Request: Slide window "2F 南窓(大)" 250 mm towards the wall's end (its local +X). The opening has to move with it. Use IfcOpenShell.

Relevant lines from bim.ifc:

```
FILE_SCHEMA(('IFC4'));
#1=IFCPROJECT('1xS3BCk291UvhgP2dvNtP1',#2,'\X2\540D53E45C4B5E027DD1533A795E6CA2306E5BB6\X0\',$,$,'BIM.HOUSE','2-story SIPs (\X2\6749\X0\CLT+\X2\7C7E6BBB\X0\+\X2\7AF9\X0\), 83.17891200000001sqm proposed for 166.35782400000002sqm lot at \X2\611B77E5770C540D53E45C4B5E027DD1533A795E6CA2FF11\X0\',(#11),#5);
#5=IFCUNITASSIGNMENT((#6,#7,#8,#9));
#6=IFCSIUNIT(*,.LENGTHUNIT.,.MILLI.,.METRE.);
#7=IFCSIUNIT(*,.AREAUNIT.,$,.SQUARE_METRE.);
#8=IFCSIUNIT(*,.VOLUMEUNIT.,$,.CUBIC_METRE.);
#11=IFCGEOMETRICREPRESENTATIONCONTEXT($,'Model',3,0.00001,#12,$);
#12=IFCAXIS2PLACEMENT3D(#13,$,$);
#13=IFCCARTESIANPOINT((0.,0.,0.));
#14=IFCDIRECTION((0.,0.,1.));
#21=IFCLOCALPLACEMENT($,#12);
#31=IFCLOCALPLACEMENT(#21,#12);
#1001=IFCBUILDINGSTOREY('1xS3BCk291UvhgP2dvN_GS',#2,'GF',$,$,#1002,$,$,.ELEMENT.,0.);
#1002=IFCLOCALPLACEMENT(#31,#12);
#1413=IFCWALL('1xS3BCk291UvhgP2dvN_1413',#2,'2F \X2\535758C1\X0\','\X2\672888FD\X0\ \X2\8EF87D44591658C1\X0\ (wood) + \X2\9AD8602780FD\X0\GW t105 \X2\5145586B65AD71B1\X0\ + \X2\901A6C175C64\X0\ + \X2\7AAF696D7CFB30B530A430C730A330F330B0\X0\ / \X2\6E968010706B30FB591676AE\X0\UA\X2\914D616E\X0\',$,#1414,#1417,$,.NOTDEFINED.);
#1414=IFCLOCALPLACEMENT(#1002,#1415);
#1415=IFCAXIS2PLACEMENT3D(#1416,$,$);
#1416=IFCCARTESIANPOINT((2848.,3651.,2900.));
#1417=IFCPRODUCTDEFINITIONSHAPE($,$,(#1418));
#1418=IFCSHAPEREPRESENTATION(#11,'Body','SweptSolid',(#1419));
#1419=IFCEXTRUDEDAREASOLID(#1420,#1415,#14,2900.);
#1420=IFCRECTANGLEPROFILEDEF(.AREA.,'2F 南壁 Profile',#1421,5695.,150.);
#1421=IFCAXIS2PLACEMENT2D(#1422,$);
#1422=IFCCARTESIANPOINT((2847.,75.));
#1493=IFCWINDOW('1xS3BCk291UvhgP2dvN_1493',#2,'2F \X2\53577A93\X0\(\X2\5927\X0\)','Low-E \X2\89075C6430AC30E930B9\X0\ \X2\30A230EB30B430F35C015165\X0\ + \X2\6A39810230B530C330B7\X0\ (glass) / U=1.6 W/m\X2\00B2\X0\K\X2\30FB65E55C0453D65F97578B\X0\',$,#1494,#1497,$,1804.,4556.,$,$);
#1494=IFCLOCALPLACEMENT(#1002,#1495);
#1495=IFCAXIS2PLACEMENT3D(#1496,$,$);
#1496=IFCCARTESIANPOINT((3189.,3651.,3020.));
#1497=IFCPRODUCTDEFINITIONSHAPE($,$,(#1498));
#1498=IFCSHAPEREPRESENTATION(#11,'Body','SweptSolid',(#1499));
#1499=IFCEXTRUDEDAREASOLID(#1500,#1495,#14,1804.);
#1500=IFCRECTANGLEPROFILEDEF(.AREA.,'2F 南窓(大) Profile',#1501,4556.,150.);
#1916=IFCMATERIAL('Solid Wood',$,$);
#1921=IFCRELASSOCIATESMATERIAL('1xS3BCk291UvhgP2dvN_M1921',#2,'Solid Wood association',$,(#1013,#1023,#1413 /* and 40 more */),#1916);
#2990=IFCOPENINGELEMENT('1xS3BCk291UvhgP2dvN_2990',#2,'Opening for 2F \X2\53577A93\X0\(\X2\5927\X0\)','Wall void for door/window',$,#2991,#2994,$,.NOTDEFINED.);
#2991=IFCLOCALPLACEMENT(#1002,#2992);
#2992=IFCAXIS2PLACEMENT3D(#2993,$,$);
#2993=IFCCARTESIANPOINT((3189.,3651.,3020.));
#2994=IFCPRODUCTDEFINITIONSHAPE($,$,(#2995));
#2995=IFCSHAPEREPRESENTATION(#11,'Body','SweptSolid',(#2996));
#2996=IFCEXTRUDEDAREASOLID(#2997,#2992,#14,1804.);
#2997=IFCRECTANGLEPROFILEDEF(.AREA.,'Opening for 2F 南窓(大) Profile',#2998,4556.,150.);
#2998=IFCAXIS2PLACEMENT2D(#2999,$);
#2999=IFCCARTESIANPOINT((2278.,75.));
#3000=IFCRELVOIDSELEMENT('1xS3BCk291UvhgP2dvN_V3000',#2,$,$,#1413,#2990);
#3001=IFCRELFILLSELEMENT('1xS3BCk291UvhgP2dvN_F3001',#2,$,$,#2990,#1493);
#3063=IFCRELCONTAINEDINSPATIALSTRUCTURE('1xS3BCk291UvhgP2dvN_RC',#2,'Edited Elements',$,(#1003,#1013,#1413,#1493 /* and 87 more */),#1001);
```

```python
import ifcopenshell
import ifcopenshell.api.geometry
import ifcopenshell.util.placement
import ifcopenshell.util.unit

model = ifcopenshell.open("bim.ifc")
unit_scale = ifcopenshell.util.unit.calculate_unit_scale(model)

window = model.by_guid("1xS3BCk291UvhgP2dvN_1493")
opening = window.FillsVoids[0].RelatingOpeningElement
wall = opening.VoidsElements[0].RelatingBuildingElement

wall_matrix = ifcopenshell.util.placement.get_local_placement(wall.ObjectPlacement)
shift = wall_matrix[:3, 0] * 0.25 / unit_scale
before = ifcopenshell.util.placement.get_local_placement(window.ObjectPlacement)[:3, 3].copy()

# The window is not placed relative to its opening, so move both.
for product in (opening, window):
    matrix = ifcopenshell.util.placement.get_local_placement(product.ObjectPlacement)
    matrix[:3, 3] += shift
    ifcopenshell.api.geometry.edit_object_placement(model, product=product, matrix=matrix, is_si=False)

after = ifcopenshell.util.placement.get_local_placement(window.ObjectPlacement)[:3, 3]
print("window moved by", (after - before).round(3) + 0.0)

model.write("bim_updated.ifc")
```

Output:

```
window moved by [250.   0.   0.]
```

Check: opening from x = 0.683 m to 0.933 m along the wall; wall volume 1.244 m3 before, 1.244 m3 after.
